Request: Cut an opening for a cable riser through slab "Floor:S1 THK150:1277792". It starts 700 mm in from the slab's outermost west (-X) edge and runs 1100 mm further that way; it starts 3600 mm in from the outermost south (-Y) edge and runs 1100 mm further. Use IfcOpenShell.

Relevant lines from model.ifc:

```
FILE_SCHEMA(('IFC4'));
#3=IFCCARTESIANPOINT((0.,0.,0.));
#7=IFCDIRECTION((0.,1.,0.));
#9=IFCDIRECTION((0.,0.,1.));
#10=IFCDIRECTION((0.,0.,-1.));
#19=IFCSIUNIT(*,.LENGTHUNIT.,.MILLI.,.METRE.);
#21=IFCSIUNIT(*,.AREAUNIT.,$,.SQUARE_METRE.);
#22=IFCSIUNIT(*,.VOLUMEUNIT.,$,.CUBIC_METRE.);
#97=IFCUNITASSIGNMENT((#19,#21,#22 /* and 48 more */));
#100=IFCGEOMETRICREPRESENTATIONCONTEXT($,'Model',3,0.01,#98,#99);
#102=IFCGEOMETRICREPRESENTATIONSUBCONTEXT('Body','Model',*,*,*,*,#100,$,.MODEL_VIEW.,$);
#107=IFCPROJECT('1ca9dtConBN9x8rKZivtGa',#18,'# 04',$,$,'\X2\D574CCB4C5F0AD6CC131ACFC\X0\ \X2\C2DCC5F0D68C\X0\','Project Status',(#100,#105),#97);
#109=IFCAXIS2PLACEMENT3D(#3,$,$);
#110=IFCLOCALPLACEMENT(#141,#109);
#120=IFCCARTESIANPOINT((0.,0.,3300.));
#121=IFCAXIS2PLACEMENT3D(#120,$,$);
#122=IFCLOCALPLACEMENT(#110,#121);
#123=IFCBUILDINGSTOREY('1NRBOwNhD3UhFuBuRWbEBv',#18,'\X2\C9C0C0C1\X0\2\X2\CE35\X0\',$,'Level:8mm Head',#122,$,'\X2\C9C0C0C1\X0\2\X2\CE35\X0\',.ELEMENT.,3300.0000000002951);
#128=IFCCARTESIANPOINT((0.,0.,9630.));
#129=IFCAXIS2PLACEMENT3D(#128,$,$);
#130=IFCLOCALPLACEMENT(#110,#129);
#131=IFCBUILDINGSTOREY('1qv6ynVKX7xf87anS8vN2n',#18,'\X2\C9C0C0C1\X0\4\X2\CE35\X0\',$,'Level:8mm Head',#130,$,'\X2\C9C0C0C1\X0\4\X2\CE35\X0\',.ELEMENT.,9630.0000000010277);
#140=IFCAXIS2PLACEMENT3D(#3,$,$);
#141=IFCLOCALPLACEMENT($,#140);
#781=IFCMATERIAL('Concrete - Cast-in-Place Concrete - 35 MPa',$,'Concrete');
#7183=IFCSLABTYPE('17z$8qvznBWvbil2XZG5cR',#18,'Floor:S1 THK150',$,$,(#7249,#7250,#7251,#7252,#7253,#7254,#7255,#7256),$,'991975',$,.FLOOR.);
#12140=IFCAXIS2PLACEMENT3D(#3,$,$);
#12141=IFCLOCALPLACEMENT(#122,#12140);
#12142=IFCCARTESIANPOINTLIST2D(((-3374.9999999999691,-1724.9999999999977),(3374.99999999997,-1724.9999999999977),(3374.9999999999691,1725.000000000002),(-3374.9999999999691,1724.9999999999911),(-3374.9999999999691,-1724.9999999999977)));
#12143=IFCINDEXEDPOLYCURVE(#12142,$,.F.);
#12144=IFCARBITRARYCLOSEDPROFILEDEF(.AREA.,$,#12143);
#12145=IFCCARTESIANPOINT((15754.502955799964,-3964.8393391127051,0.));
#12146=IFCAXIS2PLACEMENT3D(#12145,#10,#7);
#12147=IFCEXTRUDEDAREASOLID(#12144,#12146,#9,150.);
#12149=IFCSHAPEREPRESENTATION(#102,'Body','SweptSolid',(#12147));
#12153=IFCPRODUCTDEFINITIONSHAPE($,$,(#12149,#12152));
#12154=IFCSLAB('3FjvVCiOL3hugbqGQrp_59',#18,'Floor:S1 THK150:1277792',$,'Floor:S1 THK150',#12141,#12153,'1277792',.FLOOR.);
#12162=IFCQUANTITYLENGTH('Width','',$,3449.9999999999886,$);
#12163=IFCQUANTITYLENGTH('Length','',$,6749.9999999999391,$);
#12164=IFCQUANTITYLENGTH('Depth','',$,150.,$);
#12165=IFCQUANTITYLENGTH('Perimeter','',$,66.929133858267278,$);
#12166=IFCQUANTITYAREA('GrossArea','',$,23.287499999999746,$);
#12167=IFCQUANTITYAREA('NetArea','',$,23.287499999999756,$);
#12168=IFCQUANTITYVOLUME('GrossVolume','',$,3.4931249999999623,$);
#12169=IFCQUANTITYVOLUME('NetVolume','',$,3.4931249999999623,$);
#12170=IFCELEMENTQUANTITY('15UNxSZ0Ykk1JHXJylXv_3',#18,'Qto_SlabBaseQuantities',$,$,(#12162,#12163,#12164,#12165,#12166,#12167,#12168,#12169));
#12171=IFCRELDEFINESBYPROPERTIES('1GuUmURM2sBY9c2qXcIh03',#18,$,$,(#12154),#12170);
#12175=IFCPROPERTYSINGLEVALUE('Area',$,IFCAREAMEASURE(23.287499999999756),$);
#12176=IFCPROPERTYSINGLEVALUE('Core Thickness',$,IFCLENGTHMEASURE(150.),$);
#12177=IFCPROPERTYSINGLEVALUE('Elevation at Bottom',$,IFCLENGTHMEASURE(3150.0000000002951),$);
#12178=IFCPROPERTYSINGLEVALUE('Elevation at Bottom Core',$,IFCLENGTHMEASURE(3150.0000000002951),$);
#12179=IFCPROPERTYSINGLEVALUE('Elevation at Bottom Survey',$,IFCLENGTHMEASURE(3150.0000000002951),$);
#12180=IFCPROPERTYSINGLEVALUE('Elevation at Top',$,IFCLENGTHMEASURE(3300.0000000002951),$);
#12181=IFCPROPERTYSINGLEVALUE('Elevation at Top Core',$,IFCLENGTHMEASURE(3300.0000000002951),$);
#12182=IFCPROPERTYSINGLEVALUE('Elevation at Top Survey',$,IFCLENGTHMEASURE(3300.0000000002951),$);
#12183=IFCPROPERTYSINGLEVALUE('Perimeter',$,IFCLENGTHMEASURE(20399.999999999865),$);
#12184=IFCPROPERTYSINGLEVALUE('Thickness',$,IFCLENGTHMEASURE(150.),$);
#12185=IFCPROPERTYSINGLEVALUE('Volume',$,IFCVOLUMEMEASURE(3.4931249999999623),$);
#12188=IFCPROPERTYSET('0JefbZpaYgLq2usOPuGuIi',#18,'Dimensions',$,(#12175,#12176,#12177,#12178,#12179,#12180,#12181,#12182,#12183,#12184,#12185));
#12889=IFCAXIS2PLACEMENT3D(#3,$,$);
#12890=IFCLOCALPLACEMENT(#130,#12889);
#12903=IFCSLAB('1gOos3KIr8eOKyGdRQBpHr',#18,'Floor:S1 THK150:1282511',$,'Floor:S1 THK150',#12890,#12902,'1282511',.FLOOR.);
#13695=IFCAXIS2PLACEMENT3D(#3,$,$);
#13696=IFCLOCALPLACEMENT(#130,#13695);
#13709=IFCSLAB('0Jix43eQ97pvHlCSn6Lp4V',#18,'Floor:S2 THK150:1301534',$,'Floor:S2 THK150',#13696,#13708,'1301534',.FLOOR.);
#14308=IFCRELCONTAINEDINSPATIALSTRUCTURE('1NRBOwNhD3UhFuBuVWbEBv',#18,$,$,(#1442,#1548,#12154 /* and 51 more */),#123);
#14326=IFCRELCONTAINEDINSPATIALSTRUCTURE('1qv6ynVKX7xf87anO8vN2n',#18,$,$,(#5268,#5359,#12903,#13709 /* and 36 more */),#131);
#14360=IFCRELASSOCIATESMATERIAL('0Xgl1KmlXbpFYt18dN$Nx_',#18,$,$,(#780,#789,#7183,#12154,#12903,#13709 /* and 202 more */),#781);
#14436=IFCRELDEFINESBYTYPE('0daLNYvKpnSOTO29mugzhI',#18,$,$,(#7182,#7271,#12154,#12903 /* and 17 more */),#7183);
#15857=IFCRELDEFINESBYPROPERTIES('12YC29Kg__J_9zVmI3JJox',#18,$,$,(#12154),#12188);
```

```python
import numpy as np
import ifcopenshell
import ifcopenshell.api.feature
import ifcopenshell.api.geometry
import ifcopenshell.api.pset
import ifcopenshell.api.root
import ifcopenshell.geom
import ifcopenshell.util.element
import ifcopenshell.util.placement
import ifcopenshell.util.representation
import ifcopenshell.util.shape
import ifcopenshell.util.unit

model = ifcopenshell.open("model.ifc")
unit_scale = ifcopenshell.util.unit.calculate_unit_scale(model)
area_scale = ifcopenshell.util.unit.calculate_unit_scale(model, "AREAUNIT")
volume_scale = ifcopenshell.util.unit.calculate_unit_scale(model, "VOLUMEUNIT")
settings = ifcopenshell.geom.settings()


def volume(element):
    """Net volume in cubic metres, openings subtracted."""
    shape = ifcopenshell.geom.create_shape(settings, element)
    return ifcopenshell.util.shape.get_volume(shape.geometry)


slab = model.by_guid("3FjvVCiOL3hugbqGQrp_59")
before = volume(slab)

# Extent in the slab's own axes, in metres. The edges named are its -X and -Y sides.
slab_shape = ifcopenshell.geom.create_shape(settings, slab)
vertices = ifcopenshell.util.shape.get_vertices(slab_shape.geometry)
x_min, y_min, bottom = vertices.min(axis=0)
top = vertices[:, 2].max()

opening = ifcopenshell.api.root.create_entity(model, ifc_class="IfcOpeningElement", name="Cable riser opening", predefined_type="OPENING")
context = ifcopenshell.util.representation.get_context(model, "Model", "Body", "MODEL_VIEW")
width, depth = 1.1, 1.1
outline = [(0.0, 0.0), (width, 0.0), (width, depth), (0.0, depth), (0.0, 0.0)]
# Overshoot both faces by 50 mm so the cut is clean.
shape = ifcopenshell.api.geometry.add_slab_representation(
    model, context=context, depth=top - bottom + 0.1, polyline=outline
)
ifcopenshell.api.geometry.assign_representation(model, product=opening, representation=shape)

matrix = ifcopenshell.util.placement.get_local_placement(slab.ObjectPlacement)
matrix[:, 3] = matrix @ np.append(np.array([x_min + 0.7, y_min + 3.6, bottom - 0.05]) / unit_scale, 1.0)
ifcopenshell.api.geometry.edit_object_placement(model, product=opening, matrix=matrix, is_si=False)
ifcopenshell.api.feature.add_feature(model, feature=opening, element=slab)

after = volume(slab)

# Update the slab's stored quantities.
qto = model.by_id(ifcopenshell.util.element.get_pset(slab, "Qto_SlabBaseQuantities", should_inherit=False)["id"])
ifcopenshell.api.pset.edit_qto(model, qto=qto, properties={
    "NetArea": after / (top - bottom) / area_scale,
    "NetVolume": after / volume_scale,
})
pset = model.by_id(ifcopenshell.util.element.get_pset(slab, "Dimensions", should_inherit=False)["id"])
ifcopenshell.api.pset.edit_pset(model, pset=pset, properties={
    "Area": model.create_entity("IfcAreaMeasure", after / (top - bottom) / area_scale),
    "Volume": model.create_entity("IfcVolumeMeasure", after / volume_scale),
})

print(f"slab volume {before:.3f} -> {after:.3f} m3")

model.write("model_v2.ifc")
```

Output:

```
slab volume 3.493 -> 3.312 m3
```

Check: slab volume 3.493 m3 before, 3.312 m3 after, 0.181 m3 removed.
